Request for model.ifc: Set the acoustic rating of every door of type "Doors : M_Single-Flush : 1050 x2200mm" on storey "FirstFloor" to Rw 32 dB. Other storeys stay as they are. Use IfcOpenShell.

First a look at what the model holds.

```python
import ifcopenshell
import ifcopenshell.util.element

model = ifcopenshell.open("model.ifc")
print(model.schema)
storey = next(s for s in model.by_type("IfcBuildingStorey") if s.Name == "FirstFloor")
doors = [e for e in ifcopenshell.util.element.get_decomposition(storey) if e.is_a("IfcDoor")]
seen = {}
for e in doors:
    element_type = ifcopenshell.util.element.get_type(e)
    key = (element_type.Name if element_type != e and element_type else None, ifcopenshell.util.element.get_pset(e, "Pset_DoorCommon", "AcousticRating"))
    seen[key] = seen.get(key, 0) + 1
for (name, value), count in sorted(seen.items(), key=str):
    print(count, "x", name, "|", value)
```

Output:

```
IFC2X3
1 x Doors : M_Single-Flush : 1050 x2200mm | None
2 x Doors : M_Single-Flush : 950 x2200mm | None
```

```python
import ifcopenshell
import ifcopenshell.api.pset
import ifcopenshell.util.element

model = ifcopenshell.open("model.ifc")

storey = next(s for s in model.by_type("IfcBuildingStorey") if s.Name == "FirstFloor")
doors = [e for e in ifcopenshell.util.element.get_decomposition(storey) if e.is_a("IfcDoor")]

count = 0
for e in doors:
    element_type = ifcopenshell.util.element.get_type(e)
    if element_type in (None, e) or element_type.Name != "Doors : M_Single-Flush : 1050 x2200mm":
        continue
    # add_pset returns the element's existing set when there is one.
    pset = ifcopenshell.api.pset.add_pset(model, product=e, name="Pset_DoorCommon")
    ifcopenshell.api.pset.edit_pset(model, pset=pset, properties={"AcousticRating": "Rw 32 dB"})
    count += 1

print(count, "doors updated")

model.write("model_rev.ifc")
```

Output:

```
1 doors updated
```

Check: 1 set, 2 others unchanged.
